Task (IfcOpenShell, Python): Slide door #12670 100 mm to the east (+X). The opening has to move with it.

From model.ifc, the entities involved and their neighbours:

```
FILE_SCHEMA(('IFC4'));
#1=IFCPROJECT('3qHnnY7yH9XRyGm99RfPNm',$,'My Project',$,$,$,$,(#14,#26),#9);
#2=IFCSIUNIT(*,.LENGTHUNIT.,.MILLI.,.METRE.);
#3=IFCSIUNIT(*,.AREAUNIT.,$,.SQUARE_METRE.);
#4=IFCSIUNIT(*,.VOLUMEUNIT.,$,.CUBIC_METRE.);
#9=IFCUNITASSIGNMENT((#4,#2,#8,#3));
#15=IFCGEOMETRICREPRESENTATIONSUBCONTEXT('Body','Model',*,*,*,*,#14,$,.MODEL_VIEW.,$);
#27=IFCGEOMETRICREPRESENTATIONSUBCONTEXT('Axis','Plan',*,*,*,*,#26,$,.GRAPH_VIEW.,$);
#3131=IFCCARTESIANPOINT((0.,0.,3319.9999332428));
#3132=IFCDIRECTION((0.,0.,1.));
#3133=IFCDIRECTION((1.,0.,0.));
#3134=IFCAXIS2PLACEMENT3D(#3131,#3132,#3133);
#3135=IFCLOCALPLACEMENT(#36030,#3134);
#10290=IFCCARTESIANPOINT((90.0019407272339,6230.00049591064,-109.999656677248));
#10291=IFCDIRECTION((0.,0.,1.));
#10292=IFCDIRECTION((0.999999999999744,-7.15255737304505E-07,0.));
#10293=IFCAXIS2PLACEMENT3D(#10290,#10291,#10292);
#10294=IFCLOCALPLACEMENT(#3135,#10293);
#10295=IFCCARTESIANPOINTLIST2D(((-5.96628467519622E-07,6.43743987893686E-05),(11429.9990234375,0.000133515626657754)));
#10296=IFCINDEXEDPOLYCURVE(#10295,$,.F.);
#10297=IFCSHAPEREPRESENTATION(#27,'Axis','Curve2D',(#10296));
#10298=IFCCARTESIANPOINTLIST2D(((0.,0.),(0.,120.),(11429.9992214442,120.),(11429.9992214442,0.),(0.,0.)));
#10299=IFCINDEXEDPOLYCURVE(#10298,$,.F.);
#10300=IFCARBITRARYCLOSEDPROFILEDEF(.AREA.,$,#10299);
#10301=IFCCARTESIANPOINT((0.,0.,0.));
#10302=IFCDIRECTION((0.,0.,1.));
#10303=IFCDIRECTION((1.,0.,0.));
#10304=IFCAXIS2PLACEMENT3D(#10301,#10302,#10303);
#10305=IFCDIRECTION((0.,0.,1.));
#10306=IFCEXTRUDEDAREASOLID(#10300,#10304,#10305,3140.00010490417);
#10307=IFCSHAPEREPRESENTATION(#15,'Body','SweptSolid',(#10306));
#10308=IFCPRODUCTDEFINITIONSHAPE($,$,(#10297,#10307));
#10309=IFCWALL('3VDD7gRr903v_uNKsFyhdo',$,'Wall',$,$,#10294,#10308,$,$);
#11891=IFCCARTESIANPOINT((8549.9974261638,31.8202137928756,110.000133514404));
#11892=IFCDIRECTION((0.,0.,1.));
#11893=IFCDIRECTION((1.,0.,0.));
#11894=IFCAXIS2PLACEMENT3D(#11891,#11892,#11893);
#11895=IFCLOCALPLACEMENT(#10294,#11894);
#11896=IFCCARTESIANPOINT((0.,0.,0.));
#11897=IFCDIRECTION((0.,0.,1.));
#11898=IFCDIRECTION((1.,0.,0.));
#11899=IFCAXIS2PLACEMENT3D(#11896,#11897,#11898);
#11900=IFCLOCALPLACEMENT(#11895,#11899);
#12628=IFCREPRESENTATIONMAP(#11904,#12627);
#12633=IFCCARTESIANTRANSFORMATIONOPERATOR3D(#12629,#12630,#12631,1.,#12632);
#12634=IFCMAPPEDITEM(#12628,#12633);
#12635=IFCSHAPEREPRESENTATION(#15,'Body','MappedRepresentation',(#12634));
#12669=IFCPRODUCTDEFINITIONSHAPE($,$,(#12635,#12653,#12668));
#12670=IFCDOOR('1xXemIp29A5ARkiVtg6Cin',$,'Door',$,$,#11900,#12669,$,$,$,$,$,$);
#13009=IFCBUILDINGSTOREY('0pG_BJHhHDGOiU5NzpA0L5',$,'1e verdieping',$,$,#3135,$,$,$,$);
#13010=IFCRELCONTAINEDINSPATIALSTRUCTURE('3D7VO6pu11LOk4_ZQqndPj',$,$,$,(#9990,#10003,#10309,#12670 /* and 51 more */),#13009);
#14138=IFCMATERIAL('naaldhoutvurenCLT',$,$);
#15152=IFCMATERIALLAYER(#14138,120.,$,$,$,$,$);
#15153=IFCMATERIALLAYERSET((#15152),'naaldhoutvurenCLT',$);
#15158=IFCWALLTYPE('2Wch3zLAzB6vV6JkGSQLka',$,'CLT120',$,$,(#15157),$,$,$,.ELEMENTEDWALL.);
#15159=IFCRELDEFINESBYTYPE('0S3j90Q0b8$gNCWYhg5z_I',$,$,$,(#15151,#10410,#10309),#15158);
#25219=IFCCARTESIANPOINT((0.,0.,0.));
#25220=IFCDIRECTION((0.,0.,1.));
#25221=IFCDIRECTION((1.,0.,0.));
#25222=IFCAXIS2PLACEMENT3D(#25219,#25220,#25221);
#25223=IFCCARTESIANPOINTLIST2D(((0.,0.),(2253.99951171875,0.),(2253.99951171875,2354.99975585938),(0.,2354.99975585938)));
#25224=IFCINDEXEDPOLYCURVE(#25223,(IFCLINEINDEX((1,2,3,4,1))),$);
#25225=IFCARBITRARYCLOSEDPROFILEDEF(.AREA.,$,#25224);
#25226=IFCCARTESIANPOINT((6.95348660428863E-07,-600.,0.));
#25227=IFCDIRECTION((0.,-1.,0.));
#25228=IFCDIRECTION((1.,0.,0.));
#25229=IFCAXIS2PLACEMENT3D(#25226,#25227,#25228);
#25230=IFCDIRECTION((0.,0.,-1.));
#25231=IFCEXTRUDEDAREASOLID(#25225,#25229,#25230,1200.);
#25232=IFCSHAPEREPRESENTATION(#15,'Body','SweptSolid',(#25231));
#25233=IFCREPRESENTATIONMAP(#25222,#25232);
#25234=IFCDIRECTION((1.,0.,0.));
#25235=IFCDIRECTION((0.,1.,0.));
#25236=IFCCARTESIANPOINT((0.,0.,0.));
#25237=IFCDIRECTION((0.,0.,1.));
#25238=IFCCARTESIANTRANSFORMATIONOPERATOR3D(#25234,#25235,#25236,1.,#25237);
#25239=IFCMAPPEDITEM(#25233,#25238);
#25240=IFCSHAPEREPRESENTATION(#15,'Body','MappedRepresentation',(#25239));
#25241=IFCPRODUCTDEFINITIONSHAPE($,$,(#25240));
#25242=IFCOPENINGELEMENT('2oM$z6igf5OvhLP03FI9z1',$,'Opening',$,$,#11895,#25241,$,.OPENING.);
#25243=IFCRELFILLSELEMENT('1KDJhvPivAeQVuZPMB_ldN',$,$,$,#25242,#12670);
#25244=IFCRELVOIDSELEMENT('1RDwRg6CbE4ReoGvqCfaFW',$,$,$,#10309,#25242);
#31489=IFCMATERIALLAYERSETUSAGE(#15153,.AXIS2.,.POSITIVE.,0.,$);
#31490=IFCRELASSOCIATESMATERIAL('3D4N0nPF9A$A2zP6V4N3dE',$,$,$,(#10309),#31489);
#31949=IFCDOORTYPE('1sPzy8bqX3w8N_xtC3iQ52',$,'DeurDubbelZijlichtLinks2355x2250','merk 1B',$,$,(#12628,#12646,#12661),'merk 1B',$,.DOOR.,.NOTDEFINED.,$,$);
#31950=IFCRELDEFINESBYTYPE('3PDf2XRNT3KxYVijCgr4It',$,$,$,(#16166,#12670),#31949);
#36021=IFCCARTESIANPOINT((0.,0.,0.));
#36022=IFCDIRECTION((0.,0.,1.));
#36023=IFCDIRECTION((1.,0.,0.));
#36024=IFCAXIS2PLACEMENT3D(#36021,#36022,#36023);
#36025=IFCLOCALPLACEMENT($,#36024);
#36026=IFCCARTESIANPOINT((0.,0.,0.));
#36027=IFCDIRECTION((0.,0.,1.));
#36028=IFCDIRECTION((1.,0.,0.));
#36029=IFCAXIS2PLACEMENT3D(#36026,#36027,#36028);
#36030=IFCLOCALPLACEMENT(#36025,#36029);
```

```python
import ifcopenshell
import ifcopenshell.api.geometry
import ifcopenshell.util.placement

model = ifcopenshell.open("model.ifc")

door = model.by_guid("1xXemIp29A5ARkiVtg6Cin")
opening = door.FillsVoids[0].RelatingOpeningElement
wall = opening.VoidsElements[0].RelatingBuildingElement

wall_matrix = ifcopenshell.util.placement.get_local_placement(wall.ObjectPlacement)
shift = wall_matrix[:3, 0] * 100.0
before = ifcopenshell.util.placement.get_local_placement(door.ObjectPlacement)[:3, 3].copy()

# The door is placed relative to its opening, so it follows when the opening moves.
matrix = ifcopenshell.util.placement.get_local_placement(opening.ObjectPlacement)
matrix[:3, 3] += shift
ifcopenshell.api.geometry.edit_object_placement(
    model, product=opening, matrix=matrix, is_si=False, should_transform_children=True
)

after = ifcopenshell.util.placement.get_local_placement(door.ObjectPlacement)[:3, 3]
print("door moved by", (after - before).round(3) + 0.0)

model.write("model_rev.ifc")
```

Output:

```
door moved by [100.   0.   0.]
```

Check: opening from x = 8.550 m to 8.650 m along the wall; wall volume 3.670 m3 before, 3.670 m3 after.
